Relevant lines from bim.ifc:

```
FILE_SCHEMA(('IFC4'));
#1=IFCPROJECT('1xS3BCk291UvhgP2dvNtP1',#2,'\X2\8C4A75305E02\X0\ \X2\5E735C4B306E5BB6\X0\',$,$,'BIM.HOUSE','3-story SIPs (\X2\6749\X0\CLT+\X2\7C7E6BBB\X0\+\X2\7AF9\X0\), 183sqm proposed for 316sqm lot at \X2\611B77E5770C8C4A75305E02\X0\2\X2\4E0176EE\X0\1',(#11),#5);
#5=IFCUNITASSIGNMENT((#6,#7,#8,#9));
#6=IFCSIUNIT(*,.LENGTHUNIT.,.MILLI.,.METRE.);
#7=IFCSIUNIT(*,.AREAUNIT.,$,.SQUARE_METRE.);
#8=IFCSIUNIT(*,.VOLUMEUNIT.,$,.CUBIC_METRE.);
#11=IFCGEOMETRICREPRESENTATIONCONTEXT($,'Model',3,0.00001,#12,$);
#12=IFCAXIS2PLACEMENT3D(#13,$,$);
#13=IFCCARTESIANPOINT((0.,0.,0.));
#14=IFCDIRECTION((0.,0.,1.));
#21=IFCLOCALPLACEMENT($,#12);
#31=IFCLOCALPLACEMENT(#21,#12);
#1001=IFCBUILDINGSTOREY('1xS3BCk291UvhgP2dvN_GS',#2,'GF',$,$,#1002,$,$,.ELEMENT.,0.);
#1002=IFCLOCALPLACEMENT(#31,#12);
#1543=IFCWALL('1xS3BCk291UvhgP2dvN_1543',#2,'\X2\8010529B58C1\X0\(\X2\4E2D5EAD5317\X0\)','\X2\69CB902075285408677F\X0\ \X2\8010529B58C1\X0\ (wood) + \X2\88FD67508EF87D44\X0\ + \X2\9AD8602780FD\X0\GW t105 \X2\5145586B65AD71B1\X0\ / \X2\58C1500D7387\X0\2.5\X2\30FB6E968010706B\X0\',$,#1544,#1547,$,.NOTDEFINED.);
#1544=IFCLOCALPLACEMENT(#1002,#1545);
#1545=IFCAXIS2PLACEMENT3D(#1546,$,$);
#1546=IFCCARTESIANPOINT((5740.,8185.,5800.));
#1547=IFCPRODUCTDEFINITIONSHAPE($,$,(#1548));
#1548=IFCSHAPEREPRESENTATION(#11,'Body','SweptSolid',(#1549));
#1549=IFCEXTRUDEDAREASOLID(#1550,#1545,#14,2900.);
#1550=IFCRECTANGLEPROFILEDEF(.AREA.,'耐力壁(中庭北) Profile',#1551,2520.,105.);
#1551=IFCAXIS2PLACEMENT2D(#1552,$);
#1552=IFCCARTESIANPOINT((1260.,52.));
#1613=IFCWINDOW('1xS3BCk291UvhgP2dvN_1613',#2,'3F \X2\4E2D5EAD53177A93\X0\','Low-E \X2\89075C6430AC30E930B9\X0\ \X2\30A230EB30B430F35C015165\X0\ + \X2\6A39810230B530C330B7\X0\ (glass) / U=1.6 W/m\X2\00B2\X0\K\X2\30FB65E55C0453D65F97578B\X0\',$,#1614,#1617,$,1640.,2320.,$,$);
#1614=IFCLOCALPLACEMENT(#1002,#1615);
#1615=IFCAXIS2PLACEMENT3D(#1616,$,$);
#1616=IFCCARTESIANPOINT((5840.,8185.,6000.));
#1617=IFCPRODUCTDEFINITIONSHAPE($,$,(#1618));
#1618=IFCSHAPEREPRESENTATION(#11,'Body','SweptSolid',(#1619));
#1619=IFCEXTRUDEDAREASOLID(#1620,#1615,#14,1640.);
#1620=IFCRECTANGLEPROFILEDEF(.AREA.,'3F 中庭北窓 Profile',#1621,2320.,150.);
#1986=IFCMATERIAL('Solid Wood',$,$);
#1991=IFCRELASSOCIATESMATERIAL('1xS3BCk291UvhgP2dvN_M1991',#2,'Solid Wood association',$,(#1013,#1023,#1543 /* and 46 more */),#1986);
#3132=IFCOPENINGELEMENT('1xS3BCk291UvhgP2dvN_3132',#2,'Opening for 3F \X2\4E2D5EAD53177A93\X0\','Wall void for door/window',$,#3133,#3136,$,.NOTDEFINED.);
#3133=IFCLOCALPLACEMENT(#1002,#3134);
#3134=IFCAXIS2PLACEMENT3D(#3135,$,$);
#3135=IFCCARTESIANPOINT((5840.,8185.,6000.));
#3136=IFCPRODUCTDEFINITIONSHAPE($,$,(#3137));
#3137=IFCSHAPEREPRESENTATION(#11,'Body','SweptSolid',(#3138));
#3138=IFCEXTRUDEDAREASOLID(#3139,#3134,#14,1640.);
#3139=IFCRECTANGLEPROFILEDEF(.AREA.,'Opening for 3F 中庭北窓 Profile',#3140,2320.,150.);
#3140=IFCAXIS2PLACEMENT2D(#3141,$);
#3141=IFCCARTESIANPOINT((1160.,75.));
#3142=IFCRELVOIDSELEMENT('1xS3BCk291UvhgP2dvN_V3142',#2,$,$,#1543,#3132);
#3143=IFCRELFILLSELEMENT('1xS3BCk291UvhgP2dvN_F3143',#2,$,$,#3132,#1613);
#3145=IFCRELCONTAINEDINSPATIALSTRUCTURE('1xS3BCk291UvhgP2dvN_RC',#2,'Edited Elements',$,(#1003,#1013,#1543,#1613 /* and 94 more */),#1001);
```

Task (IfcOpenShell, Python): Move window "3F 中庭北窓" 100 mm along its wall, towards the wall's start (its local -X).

```python
import ifcopenshell
import ifcopenshell.api.geometry
import ifcopenshell.util.placement

model = ifcopenshell.open("bim.ifc")

window = model.by_id(1613)
opening = window.FillsVoids[0].RelatingOpeningElement
wall = opening.VoidsElements[0].RelatingBuildingElement

wall_matrix = ifcopenshell.util.placement.get_local_placement(wall.ObjectPlacement)
shift = wall_matrix[:3, 0] * -100.0
before = ifcopenshell.util.placement.get_local_placement(window.ObjectPlacement)[:3, 3].copy()

# The window is not placed relative to its opening, so move both.
for product in (opening, window):
    matrix = ifcopenshell.util.placement.get_local_placement(product.ObjectPlacement)
    matrix[:3, 3] += shift
    ifcopenshell.api.geometry.edit_object_placement(model, product=product, matrix=matrix, is_si=False)

after = ifcopenshell.util.placement.get_local_placement(window.ObjectPlacement)[:3, 3]
print("window moved by", (after - before).round(3) + 0.0)

model.write("bim_rev.ifc")
```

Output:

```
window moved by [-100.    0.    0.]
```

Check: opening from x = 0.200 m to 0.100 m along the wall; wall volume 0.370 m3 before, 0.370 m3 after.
